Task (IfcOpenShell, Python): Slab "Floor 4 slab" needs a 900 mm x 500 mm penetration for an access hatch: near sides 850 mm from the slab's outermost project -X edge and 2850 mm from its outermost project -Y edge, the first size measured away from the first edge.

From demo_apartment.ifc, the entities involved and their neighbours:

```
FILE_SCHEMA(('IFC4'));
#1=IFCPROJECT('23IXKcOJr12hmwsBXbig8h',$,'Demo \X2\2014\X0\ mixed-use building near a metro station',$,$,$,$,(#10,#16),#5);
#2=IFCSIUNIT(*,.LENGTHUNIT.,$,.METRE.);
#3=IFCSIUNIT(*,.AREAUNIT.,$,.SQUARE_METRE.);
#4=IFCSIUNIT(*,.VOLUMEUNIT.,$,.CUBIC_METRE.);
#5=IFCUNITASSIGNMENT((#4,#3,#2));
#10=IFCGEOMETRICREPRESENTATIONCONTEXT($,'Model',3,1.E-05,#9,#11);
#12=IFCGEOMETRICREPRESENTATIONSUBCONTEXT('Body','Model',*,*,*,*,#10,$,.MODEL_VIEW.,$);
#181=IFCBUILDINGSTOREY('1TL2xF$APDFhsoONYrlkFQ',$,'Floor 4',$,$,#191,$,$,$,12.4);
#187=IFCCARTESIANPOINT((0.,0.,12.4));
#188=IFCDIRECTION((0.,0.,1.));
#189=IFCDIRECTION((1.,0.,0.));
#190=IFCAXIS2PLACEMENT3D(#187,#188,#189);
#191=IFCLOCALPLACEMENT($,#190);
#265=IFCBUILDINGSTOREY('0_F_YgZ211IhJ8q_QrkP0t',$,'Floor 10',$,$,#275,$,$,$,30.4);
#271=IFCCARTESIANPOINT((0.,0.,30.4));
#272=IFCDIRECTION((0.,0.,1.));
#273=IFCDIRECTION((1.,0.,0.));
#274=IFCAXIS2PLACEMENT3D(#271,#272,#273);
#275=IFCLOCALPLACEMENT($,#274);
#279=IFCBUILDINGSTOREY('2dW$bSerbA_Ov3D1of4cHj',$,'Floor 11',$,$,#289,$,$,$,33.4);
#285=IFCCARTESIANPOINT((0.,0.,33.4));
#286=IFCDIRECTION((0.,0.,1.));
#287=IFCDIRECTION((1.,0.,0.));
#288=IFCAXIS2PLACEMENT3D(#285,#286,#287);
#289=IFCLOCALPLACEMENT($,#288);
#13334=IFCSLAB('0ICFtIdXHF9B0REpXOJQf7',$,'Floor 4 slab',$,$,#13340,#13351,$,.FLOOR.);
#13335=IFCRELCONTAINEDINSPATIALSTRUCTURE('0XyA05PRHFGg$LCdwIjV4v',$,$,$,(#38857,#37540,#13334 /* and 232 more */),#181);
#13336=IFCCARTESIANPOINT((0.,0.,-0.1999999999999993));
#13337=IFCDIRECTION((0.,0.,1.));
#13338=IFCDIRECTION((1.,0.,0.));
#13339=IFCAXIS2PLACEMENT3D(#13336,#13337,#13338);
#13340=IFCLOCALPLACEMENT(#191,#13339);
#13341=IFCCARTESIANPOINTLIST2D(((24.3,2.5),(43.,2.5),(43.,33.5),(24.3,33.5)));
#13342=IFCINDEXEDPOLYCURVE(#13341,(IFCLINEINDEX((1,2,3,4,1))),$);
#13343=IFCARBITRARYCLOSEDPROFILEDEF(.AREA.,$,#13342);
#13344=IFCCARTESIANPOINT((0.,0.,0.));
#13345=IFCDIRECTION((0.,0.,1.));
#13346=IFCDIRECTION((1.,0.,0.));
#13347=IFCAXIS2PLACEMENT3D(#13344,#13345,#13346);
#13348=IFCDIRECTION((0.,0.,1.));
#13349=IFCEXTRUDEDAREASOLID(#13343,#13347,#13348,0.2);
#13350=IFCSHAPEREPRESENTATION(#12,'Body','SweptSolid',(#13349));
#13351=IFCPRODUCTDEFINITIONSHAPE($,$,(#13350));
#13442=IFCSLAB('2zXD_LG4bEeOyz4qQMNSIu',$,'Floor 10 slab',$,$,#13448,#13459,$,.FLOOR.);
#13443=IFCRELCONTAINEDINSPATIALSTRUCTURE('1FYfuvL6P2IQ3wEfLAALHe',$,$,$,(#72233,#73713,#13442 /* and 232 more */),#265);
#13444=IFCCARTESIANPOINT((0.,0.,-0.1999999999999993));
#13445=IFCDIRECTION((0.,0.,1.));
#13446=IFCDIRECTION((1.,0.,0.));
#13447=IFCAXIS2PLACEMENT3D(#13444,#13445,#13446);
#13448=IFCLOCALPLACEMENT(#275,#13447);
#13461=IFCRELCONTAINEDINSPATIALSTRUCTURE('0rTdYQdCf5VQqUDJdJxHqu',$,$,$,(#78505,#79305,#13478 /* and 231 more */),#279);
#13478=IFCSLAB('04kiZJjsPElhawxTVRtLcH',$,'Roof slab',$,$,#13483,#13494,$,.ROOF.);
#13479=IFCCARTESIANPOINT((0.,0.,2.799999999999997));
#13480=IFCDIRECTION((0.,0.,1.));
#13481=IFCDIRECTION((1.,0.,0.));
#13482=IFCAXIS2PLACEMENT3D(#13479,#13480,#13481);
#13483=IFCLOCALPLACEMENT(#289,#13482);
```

```python
import numpy as np
import ifcopenshell
import ifcopenshell.api.feature
import ifcopenshell.api.geometry
import ifcopenshell.api.root
import ifcopenshell.geom
import ifcopenshell.util.placement
import ifcopenshell.util.representation
import ifcopenshell.util.shape
import ifcopenshell.util.unit

model = ifcopenshell.open("demo_apartment.ifc")
unit_scale = ifcopenshell.util.unit.calculate_unit_scale(model)
settings = ifcopenshell.geom.settings()


def volume(element):
    """Net volume in cubic metres, openings subtracted."""
    shape = ifcopenshell.geom.create_shape(settings, element)
    return ifcopenshell.util.shape.get_volume(shape.geometry)


slab = model.by_guid("0ICFtIdXHF9B0REpXOJQf7")
before = volume(slab)

# Extent in the slab's own axes, in metres. The edges named are its -X and -Y sides.
slab_shape = ifcopenshell.geom.create_shape(settings, slab)
vertices = ifcopenshell.util.shape.get_vertices(slab_shape.geometry)
x_min, y_min, bottom = vertices.min(axis=0)
top = vertices[:, 2].max()

opening = ifcopenshell.api.root.create_entity(model, ifc_class="IfcOpeningElement", name="Access hatch opening", predefined_type="OPENING")
context = ifcopenshell.util.representation.get_context(model, "Model", "Body", "MODEL_VIEW")
width, depth = 0.9, 0.5
outline = [(0.0, 0.0), (width, 0.0), (width, depth), (0.0, depth), (0.0, 0.0)]
# Overshoot both faces by 50 mm so the cut is clean.
shape = ifcopenshell.api.geometry.add_slab_representation(
    model, context=context, depth=top - bottom + 0.1, polyline=outline
)
ifcopenshell.api.geometry.assign_representation(model, product=opening, representation=shape)

matrix = ifcopenshell.util.placement.get_local_placement(slab.ObjectPlacement)
matrix[:, 3] = matrix @ np.append(np.array([x_min + 0.85, y_min + 2.85, bottom - 0.05]) / unit_scale, 1.0)
ifcopenshell.api.geometry.edit_object_placement(model, product=opening, matrix=matrix, is_si=False)
ifcopenshell.api.feature.add_feature(model, feature=opening, element=slab)

after = volume(slab)

print(f"slab volume {before:.3f} -> {after:.3f} m3")

model.write("demo_apartment_v2.ifc")
```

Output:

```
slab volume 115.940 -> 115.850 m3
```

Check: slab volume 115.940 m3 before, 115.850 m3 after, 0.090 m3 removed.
